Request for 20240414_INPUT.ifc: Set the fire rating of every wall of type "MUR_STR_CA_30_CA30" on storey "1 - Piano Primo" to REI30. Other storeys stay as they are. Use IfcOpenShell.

First a look at what the model holds.

```python
import ifcopenshell
import ifcopenshell.util.element

model = ifcopenshell.open("20240414_INPUT.ifc")
print(model.schema)
storey = next(s for s in model.by_type("IfcBuildingStorey") if s.Name == "1 - Piano Primo")
walls = [e for e in ifcopenshell.util.element.get_decomposition(storey) if e.is_a("IfcWall")]
seen = {}
for e in walls:
    element_type = ifcopenshell.util.element.get_type(e)
    key = (element_type.Name if element_type != e and element_type else None, ifcopenshell.util.element.get_pset(e, "Pset_WallCommon", "FireRating"))
    seen[key] = seen.get(key, 0) + 1
for (name, value), count in sorted(seen.items(), key=str):
    print(count, "x", name, "|", value)
```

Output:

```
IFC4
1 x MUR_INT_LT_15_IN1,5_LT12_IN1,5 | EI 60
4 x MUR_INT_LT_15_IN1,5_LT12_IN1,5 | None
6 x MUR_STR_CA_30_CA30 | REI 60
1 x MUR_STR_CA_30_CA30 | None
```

```python
import ifcopenshell
import ifcopenshell.api.pset
import ifcopenshell.util.element

model = ifcopenshell.open("20240414_INPUT.ifc")

storey = next(s for s in model.by_type("IfcBuildingStorey") if s.Name == "1 - Piano Primo")
walls = [e for e in ifcopenshell.util.element.get_decomposition(storey) if e.is_a("IfcWall")]

count = 0
for e in walls:
    element_type = ifcopenshell.util.element.get_type(e)
    if element_type in (None, e) or element_type.Name != "MUR_STR_CA_30_CA30":
        continue
    # add_pset returns the element's existing set when there is one.
    pset = ifcopenshell.api.pset.add_pset(model, product=e, name="Pset_WallCommon")
    ifcopenshell.api.pset.edit_pset(model, pset=pset, properties={"FireRating": "REI30"})
    count += 1

print(count, "walls updated")

model.write("20240414_INPUT_rev.ifc")
```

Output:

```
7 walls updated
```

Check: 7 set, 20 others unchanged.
